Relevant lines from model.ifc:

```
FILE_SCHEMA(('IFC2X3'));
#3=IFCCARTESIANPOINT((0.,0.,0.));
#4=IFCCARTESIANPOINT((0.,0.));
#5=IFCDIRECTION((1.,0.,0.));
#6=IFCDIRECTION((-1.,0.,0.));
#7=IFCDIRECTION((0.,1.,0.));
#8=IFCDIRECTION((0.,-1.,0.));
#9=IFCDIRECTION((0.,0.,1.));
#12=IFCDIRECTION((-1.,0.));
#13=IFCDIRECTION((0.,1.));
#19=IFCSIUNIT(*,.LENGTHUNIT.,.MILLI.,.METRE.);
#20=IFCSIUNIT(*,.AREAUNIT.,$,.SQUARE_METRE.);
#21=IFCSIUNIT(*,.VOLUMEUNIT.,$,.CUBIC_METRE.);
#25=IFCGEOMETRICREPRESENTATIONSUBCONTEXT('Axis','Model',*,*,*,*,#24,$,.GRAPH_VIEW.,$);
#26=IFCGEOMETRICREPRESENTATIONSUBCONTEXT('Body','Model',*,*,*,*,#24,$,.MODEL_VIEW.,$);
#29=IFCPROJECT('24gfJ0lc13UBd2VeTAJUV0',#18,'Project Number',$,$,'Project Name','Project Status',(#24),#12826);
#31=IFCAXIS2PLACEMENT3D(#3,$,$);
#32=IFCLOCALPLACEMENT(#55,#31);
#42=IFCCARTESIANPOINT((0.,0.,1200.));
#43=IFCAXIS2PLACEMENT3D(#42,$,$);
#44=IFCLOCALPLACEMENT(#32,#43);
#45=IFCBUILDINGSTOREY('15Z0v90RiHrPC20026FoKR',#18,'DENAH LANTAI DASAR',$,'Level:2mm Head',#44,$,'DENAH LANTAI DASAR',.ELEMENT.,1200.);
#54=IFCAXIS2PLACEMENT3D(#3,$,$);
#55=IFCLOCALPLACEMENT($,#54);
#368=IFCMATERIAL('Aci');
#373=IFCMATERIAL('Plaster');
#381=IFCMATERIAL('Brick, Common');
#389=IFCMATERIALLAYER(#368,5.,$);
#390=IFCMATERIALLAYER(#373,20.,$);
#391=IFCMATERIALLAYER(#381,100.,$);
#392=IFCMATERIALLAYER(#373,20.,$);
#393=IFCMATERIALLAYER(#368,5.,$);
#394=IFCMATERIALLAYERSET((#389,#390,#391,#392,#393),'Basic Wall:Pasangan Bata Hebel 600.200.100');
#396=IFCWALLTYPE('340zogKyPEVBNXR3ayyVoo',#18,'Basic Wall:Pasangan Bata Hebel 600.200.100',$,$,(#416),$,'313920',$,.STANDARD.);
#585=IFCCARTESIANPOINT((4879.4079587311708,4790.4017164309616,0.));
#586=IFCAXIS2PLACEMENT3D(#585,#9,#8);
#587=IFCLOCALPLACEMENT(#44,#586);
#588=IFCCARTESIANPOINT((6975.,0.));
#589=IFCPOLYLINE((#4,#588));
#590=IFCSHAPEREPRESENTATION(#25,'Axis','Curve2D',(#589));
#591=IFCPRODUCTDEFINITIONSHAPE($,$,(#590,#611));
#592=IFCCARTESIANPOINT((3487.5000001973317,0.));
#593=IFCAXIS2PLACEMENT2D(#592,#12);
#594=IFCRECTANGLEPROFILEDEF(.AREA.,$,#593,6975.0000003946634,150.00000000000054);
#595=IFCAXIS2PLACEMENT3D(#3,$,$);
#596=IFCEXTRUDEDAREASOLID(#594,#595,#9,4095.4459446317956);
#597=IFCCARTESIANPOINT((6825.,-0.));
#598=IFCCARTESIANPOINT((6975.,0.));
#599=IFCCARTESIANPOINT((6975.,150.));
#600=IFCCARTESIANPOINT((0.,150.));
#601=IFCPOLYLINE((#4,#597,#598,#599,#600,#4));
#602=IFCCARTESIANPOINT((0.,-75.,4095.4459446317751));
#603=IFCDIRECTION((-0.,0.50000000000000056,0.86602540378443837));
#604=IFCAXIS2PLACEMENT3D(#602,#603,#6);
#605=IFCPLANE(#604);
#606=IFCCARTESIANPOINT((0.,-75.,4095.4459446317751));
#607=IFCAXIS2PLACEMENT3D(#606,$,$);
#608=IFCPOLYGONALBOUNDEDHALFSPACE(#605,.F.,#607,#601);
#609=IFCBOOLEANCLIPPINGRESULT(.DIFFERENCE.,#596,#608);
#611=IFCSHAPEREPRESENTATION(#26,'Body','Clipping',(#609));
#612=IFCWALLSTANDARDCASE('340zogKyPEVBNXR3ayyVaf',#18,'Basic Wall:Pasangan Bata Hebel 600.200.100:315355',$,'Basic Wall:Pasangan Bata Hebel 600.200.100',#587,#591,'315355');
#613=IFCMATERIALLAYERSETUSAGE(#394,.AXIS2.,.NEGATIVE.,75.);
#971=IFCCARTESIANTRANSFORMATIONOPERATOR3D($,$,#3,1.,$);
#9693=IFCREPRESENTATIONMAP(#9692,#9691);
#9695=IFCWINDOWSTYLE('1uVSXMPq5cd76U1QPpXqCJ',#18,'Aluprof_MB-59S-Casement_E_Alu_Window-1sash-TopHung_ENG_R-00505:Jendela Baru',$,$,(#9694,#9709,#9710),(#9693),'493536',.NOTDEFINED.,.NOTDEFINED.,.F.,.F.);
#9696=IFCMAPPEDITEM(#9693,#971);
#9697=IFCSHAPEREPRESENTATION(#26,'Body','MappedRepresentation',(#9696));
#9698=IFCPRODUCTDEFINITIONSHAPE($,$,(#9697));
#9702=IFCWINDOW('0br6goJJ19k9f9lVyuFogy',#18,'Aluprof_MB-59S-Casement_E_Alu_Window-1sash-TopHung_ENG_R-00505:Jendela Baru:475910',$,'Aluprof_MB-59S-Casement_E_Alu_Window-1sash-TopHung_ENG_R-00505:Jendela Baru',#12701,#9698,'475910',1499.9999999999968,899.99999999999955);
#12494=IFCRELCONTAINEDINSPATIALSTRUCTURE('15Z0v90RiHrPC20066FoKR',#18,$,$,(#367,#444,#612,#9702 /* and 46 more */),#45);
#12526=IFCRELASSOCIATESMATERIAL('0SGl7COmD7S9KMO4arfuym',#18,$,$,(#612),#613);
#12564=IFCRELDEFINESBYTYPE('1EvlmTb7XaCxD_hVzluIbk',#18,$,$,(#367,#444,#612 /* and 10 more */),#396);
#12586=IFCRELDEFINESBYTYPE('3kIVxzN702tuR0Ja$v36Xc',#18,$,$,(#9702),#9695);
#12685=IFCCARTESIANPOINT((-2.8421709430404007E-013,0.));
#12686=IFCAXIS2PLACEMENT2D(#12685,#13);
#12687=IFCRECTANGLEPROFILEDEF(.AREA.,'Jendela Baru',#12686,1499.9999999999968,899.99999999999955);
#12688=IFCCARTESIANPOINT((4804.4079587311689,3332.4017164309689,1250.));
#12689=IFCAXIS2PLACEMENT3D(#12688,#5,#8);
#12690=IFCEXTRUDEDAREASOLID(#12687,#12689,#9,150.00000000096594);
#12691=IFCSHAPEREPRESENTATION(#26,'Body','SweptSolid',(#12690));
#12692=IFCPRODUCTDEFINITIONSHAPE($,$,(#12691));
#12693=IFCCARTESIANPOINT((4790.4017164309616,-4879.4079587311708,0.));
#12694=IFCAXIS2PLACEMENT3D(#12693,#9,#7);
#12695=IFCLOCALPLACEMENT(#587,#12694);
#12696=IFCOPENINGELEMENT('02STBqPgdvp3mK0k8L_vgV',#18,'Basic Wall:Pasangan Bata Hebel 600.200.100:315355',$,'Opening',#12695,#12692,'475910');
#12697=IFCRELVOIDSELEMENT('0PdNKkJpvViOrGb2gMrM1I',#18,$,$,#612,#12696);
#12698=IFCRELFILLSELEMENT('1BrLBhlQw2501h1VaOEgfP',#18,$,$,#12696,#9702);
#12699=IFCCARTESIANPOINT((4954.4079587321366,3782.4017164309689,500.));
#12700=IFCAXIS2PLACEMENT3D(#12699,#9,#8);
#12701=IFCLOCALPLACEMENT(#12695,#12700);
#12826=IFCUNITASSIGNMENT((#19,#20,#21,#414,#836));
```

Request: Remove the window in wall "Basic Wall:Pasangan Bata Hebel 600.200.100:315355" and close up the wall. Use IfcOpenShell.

```python
import ifcopenshell
import ifcopenshell.api.feature
import ifcopenshell.api.root
import ifcopenshell.geom
import ifcopenshell.util.shape

model = ifcopenshell.open("model.ifc")
settings = ifcopenshell.geom.settings()


def volume(element):
    """Net volume in cubic metres, openings subtracted."""
    shape = ifcopenshell.geom.create_shape(settings, element)
    return ifcopenshell.util.shape.get_volume(shape.geometry)


window = model.by_guid("0br6goJJ19k9f9lVyuFogy")
opening = window.FillsVoids[0].RelatingOpeningElement
wall = opening.VoidsElements[0].RelatingBuildingElement
before = volume(wall)

ifcopenshell.api.root.remove_product(model, product=window)
ifcopenshell.api.feature.remove_feature(model, feature=opening)

after = volume(wall)

print(f"wall volume {before:.3f} -> {after:.3f} m3")

model.write("model_edited.ifc")
```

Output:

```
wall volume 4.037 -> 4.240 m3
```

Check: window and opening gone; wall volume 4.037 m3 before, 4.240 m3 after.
